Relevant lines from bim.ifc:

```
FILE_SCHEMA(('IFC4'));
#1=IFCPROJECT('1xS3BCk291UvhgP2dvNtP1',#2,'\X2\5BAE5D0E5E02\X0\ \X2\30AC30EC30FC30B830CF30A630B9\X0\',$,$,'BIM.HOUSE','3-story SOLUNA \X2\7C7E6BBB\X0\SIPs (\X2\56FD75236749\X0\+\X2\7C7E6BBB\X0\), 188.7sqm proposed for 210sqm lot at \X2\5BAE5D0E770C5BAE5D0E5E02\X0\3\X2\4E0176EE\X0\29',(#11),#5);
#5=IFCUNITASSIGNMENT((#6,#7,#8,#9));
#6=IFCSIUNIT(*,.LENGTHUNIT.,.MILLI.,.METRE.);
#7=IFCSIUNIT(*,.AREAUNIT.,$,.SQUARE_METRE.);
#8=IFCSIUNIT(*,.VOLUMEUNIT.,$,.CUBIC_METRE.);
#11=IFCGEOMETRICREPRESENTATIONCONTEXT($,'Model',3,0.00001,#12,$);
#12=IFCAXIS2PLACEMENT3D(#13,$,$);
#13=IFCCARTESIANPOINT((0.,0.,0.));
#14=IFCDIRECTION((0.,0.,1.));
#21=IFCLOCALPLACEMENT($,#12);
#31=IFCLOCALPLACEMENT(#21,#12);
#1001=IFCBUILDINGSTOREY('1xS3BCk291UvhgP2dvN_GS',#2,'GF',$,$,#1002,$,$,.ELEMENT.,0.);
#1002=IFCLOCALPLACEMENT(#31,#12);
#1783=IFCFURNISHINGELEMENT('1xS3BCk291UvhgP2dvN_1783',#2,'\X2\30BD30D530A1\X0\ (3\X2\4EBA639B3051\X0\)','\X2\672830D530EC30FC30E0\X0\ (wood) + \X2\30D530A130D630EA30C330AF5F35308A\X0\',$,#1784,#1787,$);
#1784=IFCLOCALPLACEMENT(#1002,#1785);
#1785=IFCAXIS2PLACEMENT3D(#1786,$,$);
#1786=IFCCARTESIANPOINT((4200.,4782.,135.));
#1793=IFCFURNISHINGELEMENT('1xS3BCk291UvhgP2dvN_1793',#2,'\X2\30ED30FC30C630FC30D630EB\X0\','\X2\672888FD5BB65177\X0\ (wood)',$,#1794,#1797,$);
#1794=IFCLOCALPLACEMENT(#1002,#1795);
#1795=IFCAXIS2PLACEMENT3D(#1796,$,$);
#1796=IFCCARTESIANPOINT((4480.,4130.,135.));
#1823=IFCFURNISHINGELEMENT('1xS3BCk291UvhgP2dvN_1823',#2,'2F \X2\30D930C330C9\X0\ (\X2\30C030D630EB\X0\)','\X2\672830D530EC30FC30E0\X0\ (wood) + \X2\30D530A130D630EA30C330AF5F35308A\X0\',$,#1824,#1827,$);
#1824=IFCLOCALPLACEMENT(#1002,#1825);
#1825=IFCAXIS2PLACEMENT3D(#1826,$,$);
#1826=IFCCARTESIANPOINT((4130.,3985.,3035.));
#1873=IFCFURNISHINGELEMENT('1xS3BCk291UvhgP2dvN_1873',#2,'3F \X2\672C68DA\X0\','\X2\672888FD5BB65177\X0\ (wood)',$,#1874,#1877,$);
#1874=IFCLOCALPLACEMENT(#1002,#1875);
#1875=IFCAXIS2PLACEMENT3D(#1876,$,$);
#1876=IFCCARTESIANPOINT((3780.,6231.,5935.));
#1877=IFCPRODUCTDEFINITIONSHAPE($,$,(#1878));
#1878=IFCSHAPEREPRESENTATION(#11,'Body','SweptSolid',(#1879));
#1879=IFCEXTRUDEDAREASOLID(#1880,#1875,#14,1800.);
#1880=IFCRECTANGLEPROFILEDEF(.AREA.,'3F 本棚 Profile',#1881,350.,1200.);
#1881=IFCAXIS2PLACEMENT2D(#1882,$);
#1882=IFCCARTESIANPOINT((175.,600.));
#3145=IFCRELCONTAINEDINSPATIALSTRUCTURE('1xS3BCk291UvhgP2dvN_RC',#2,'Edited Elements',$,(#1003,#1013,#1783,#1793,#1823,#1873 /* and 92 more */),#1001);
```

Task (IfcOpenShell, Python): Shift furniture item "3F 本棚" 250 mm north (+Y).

```python
import ifcopenshell
import ifcopenshell.api.geometry
import ifcopenshell.util.placement

model = ifcopenshell.open("bim.ifc")

item = model.by_guid("1xS3BCk291UvhgP2dvN_1873")
matrix = ifcopenshell.util.placement.get_local_placement(item.ObjectPlacement)
matrix[1, 3] += 250.0
ifcopenshell.api.geometry.edit_object_placement(model, product=item, matrix=matrix, is_si=False)

print(ifcopenshell.util.placement.get_local_placement(item.ObjectPlacement).round(3) + 0.0)

model.write("bim_updated.ifc")
```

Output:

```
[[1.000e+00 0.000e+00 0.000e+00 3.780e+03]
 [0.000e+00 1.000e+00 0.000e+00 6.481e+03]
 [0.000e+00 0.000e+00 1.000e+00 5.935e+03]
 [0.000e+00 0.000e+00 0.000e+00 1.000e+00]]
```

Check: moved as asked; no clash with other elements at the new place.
